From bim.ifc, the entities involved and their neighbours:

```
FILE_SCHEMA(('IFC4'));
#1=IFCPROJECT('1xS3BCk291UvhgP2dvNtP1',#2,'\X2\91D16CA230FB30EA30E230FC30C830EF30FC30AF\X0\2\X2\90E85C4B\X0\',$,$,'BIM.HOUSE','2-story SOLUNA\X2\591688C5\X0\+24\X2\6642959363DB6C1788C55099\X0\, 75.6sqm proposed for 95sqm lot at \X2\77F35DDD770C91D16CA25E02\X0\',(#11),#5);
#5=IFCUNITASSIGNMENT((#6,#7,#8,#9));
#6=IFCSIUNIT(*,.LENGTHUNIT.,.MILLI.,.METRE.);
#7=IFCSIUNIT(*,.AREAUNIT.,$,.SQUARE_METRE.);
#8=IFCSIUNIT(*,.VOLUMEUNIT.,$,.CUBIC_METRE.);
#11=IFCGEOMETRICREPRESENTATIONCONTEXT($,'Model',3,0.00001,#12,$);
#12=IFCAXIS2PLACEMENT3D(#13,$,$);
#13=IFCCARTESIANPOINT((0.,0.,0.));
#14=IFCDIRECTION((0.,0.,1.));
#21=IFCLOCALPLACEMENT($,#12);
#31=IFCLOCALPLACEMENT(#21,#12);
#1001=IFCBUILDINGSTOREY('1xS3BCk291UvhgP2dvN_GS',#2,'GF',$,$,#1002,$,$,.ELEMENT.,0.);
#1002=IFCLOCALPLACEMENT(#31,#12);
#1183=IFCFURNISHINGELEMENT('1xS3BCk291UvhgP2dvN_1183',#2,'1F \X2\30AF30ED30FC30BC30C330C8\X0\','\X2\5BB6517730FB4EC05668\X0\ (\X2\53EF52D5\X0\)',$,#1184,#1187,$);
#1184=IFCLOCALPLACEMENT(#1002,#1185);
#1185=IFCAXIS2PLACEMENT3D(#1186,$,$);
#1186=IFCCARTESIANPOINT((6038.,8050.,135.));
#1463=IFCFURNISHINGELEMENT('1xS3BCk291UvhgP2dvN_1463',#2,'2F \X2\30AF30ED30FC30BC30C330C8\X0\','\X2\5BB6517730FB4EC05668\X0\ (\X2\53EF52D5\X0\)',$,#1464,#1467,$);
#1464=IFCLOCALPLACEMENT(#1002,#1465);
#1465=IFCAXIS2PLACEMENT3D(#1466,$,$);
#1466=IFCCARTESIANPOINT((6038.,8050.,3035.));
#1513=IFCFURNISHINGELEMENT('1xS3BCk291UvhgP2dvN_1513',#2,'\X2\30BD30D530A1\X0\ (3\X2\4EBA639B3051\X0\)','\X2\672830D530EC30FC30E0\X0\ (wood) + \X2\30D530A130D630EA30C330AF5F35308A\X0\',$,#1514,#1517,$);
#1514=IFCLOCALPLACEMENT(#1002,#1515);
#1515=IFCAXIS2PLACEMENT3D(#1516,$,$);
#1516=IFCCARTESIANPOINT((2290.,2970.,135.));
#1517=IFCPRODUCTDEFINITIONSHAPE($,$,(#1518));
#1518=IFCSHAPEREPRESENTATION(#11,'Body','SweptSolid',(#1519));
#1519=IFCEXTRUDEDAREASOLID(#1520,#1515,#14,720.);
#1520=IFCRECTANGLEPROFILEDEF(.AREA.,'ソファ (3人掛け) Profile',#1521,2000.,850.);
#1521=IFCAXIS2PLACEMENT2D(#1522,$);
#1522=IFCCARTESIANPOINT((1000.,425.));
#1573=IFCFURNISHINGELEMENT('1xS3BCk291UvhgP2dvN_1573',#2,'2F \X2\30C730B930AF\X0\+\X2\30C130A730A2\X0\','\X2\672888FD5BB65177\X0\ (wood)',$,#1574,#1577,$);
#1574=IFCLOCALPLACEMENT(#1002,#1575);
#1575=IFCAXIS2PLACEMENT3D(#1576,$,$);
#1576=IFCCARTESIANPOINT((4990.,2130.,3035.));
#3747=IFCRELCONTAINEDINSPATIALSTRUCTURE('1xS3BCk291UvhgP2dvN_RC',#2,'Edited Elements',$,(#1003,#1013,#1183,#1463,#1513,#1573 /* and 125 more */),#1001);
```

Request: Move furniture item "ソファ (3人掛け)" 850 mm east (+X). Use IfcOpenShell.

```python
import ifcopenshell
import ifcopenshell.api.geometry
import ifcopenshell.util.placement
import ifcopenshell.util.unit

model = ifcopenshell.open("bim.ifc")
unit_scale = ifcopenshell.util.unit.calculate_unit_scale(model)

item = model.by_guid("1xS3BCk291UvhgP2dvN_1513")
matrix = ifcopenshell.util.placement.get_local_placement(item.ObjectPlacement)
matrix[0, 3] += 0.85 / unit_scale
ifcopenshell.api.geometry.edit_object_placement(model, product=item, matrix=matrix, is_si=False)

print(ifcopenshell.util.placement.get_local_placement(item.ObjectPlacement).round(3) + 0.0)

model.write("bim_v2.ifc")
```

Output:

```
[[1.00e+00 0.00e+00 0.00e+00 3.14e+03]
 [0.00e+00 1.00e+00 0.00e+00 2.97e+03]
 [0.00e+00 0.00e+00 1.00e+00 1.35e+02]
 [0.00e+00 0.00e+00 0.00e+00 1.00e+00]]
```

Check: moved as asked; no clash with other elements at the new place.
